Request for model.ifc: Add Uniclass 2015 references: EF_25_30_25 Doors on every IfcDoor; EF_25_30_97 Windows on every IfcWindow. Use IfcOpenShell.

First a look at what the model holds.

```python
import ifcopenshell

model = ifcopenshell.open("model.ifc")
print(model.schema)
print("classifications:", [c.Name for c in model.by_type("IfcClassification")])
for ifc_class in ("IfcDoor", "IfcRoof", "IfcStair", "IfcWall", "IfcWindow"):
    print(ifc_class, len(model.by_type(ifc_class)))
```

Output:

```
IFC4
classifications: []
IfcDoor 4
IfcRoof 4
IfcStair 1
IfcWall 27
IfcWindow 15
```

```python
import ifcopenshell
import ifcopenshell.api.classification

model = ifcopenshell.open("model.ifc")

system = ifcopenshell.api.classification.add_classification(model, classification="Uniclass 2015")

codes = {
    "IfcDoor": ("EF_25_30_25", "Doors"),
    "IfcWindow": ("EF_25_30_97", "Windows"),
}
for ifc_class, (code, name) in codes.items():
    products = model.by_type(ifc_class)
    ifcopenshell.api.classification.add_reference(
        model, products=products, classification=system, identification=code, name=name
    )
    print(code, len(products))

model.write("model_rev.ifc")
```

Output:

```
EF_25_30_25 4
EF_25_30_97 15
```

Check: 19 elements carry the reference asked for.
